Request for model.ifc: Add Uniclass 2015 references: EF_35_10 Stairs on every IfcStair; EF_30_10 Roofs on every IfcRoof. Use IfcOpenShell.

First a look at what the model holds.

```python
import ifcopenshell

model = ifcopenshell.open("model.ifc")
print(model.schema)
print("classifications:", [c.Name for c in model.by_type("IfcClassification")])
for ifc_class in ("IfcDoor", "IfcRoof", "IfcStair", "IfcWall", "IfcWindow"):
    print(ifc_class, len(model.by_type(ifc_class)))
```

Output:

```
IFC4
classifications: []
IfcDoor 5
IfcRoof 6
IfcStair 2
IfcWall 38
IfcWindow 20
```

```python
import ifcopenshell
import ifcopenshell.api.classification

model = ifcopenshell.open("model.ifc")

system = ifcopenshell.api.classification.add_classification(model, classification="Uniclass 2015")

codes = {
    "IfcStair": ("EF_35_10", "Stairs"),
    "IfcRoof": ("EF_30_10", "Roofs"),
}
for ifc_class, (code, name) in codes.items():
    products = model.by_type(ifc_class)
    ifcopenshell.api.classification.add_reference(
        model, products=products, classification=system, identification=code, name=name
    )
    print(code, len(products))

model.write("model_rev.ifc")
```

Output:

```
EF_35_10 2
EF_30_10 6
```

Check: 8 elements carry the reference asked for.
